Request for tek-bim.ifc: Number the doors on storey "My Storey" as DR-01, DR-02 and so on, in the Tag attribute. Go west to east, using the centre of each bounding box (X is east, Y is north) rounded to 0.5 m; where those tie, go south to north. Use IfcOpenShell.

First a look at what the model holds.

```python
import ifcopenshell
import ifcopenshell.util.element
import ifcopenshell.util.placement

model = ifcopenshell.open("tek-bim.ifc")
print(model.schema)
storey = next(s for s in model.by_type("IfcBuildingStorey") if s.Name == "My Storey")
doors = [e for e in ifcopenshell.util.element.get_decomposition(storey) if e.is_a("IfcDoor")]
for e in sorted(doors, key=lambda e: e.id()):
    origin = ifcopenshell.util.placement.get_local_placement(e.ObjectPlacement)[:3, 3]
    print(e.id(), e.Tag, e.Name, origin.round(2) + 0.0, sep=" | ")
```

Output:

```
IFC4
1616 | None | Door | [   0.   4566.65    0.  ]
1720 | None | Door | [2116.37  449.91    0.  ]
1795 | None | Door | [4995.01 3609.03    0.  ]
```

```python
import ifcopenshell
import ifcopenshell.geom
import ifcopenshell.util.element
import ifcopenshell.util.shape

model = ifcopenshell.open("tek-bim.ifc")
settings = ifcopenshell.geom.settings()
settings.set("use-world-coords", True)


def centre(element):
    shape = ifcopenshell.geom.create_shape(settings, element)
    return ifcopenshell.util.shape.get_bbox_centroid(shape.geometry)


storey = next(s for s in model.by_type("IfcBuildingStorey") if s.Name == "My Storey")
doors = [e for e in ifcopenshell.util.element.get_decomposition(storey) if e.is_a("IfcDoor")]

# Insertion points can sit at a corner or the storey origin, so sort by the geometry (in metres).
centres = {e: centre(e) for e in doors}
doors.sort(key=lambda e: (round(centres[e][0] / 0.5), centres[e][1]))

for i, e in enumerate(doors, start=1):
    number = f"DR-{i:02d}"
    e.Tag = number
    print(e.id(), number)

model.write("tek-bim_updated.ifc")
```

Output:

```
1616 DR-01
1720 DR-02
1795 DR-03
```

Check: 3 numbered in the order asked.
